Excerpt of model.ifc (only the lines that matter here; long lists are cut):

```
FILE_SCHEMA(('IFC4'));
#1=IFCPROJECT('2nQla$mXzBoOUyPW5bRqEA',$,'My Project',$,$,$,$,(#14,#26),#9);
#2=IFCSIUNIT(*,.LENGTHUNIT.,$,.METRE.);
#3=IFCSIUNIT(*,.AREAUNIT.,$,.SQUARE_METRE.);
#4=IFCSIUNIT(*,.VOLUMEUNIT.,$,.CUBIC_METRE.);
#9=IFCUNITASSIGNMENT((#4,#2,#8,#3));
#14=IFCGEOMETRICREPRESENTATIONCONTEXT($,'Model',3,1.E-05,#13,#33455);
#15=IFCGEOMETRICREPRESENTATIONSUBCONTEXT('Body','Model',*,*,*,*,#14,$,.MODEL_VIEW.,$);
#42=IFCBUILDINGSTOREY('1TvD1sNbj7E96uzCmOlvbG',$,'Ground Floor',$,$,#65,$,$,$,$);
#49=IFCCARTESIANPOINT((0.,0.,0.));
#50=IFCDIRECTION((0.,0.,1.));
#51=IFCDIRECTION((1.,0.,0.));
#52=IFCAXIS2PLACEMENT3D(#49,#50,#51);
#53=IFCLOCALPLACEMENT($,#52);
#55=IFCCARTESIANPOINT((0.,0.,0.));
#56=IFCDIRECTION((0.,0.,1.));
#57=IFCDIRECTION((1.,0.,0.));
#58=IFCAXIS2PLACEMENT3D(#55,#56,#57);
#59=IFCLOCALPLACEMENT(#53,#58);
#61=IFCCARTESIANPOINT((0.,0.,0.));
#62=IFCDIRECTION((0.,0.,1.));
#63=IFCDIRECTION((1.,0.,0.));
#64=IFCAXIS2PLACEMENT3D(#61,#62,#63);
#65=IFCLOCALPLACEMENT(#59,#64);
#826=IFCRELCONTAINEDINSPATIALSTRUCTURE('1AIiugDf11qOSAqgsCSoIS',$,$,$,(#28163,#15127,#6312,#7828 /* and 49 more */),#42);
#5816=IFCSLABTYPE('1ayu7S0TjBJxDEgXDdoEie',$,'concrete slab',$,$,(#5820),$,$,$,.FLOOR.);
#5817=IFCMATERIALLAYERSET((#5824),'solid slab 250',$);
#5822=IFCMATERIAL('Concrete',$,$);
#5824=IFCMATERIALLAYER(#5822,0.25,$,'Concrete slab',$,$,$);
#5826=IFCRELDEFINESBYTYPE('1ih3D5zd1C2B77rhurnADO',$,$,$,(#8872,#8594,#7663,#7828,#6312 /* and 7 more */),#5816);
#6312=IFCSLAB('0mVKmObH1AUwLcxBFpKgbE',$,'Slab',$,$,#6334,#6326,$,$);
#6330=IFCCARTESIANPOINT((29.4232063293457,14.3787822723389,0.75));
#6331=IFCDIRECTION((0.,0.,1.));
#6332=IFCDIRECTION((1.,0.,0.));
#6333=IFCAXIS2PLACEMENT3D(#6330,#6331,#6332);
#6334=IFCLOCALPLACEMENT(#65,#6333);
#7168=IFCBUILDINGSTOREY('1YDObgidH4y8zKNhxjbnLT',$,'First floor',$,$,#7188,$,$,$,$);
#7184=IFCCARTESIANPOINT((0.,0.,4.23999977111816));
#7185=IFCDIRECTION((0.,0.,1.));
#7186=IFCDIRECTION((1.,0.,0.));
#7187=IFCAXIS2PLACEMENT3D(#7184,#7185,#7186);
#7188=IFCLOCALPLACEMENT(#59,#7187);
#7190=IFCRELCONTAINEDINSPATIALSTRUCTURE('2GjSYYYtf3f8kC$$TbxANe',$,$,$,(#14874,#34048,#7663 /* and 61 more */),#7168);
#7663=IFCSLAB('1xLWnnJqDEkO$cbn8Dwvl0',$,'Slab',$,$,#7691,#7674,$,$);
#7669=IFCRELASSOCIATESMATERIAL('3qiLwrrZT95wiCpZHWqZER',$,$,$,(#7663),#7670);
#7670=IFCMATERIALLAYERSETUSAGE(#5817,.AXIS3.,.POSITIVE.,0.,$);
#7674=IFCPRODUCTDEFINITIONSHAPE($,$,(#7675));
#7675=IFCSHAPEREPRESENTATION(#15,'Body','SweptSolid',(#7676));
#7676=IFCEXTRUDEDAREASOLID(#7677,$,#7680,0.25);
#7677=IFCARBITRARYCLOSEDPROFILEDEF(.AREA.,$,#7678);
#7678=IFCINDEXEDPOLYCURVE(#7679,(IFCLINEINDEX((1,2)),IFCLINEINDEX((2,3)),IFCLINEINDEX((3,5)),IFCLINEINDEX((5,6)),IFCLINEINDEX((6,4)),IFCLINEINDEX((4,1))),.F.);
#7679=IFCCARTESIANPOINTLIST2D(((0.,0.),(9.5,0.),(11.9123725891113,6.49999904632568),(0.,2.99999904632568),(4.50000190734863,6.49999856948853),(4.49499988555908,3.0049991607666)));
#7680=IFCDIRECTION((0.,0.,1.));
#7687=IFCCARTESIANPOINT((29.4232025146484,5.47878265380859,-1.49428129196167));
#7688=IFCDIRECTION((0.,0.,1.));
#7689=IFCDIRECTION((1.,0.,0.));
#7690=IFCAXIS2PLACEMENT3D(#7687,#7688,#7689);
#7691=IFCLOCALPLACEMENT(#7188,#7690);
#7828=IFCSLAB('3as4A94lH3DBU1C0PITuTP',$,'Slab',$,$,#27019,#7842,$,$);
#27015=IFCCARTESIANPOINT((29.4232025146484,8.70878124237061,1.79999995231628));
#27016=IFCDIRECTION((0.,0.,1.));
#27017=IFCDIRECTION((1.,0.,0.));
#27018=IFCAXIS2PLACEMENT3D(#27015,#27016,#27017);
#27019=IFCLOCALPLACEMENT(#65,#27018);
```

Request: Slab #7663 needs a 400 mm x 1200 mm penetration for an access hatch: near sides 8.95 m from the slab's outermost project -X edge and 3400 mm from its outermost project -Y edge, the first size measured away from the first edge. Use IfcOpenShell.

```python
import numpy as np
import ifcopenshell
import ifcopenshell.api.feature
import ifcopenshell.api.geometry
import ifcopenshell.api.root
import ifcopenshell.geom
import ifcopenshell.util.placement
import ifcopenshell.util.representation
import ifcopenshell.util.shape
import ifcopenshell.util.unit

model = ifcopenshell.open("model.ifc")
unit_scale = ifcopenshell.util.unit.calculate_unit_scale(model)
settings = ifcopenshell.geom.settings()


def volume(element):
    """Net volume in cubic metres, openings subtracted."""
    shape = ifcopenshell.geom.create_shape(settings, element)
    return ifcopenshell.util.shape.get_volume(shape.geometry)


slab = model.by_guid("1xLWnnJqDEkO$cbn8Dwvl0")
before = volume(slab)

# Extent in the slab's own axes, in metres. The edges named are its -X and -Y sides.
slab_shape = ifcopenshell.geom.create_shape(settings, slab)
vertices = ifcopenshell.util.shape.get_vertices(slab_shape.geometry)
x_min, y_min, bottom = vertices.min(axis=0)
top = vertices[:, 2].max()

opening = ifcopenshell.api.root.create_entity(model, ifc_class="IfcOpeningElement", name="Access hatch opening", predefined_type="OPENING")
context = ifcopenshell.util.representation.get_context(model, "Model", "Body", "MODEL_VIEW")
width, depth = 0.4, 1.2
outline = [(0.0, 0.0), (width, 0.0), (width, depth), (0.0, depth), (0.0, 0.0)]
# Overshoot both faces by 50 mm so the cut is clean.
shape = ifcopenshell.api.geometry.add_slab_representation(
    model, context=context, depth=top - bottom + 0.1, polyline=outline
)
ifcopenshell.api.geometry.assign_representation(model, product=opening, representation=shape)

matrix = ifcopenshell.util.placement.get_local_placement(slab.ObjectPlacement)
matrix[:, 3] = matrix @ np.append(np.array([x_min + 8.95, y_min + 3.4, bottom - 0.05]) / unit_scale, 1.0)
ifcopenshell.api.geometry.edit_object_placement(model, product=opening, matrix=matrix, is_si=False)
ifcopenshell.api.feature.add_feature(model, feature=opening, element=slab)

after = volume(slab)

print(f"slab volume {before:.3f} -> {after:.3f} m3")

model.write("model_edited.ifc")
```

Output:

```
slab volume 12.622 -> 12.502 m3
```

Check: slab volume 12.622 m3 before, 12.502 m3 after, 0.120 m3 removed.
